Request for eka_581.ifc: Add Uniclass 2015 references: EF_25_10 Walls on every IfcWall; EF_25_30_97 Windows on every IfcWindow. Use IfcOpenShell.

First a look at what the model holds.

```python
import ifcopenshell

model = ifcopenshell.open("eka_581.ifc")
print(model.schema)
print("classifications:", [c.Name for c in model.by_type("IfcClassification")])
for ifc_class in ("IfcDoor", "IfcRoof", "IfcStair", "IfcWall", "IfcWindow"):
    print(ifc_class, len(model.by_type(ifc_class)))
```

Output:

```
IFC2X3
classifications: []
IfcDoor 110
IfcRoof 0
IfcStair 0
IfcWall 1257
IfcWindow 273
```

```python
import ifcopenshell
import ifcopenshell.api.classification

model = ifcopenshell.open("eka_581.ifc")

# IFC2X3 requires Source and Edition and has no link from the project to the system.
system = model.create_entity("IfcClassification", Source="NBS", Edition="2015", Name="Uniclass 2015")

codes = {
    "IfcWall": ("EF_25_10", "Walls"),
    "IfcWindow": ("EF_25_30_97", "Windows"),
}
for ifc_class, (code, name) in codes.items():
    products = model.by_type(ifc_class)
    ifcopenshell.api.classification.add_reference(
        model, products=products, classification=system, identification=code, name=name
    )
    print(code, len(products))

model.write("eka_581-out.ifc")
```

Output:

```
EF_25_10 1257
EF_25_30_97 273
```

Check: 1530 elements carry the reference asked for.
